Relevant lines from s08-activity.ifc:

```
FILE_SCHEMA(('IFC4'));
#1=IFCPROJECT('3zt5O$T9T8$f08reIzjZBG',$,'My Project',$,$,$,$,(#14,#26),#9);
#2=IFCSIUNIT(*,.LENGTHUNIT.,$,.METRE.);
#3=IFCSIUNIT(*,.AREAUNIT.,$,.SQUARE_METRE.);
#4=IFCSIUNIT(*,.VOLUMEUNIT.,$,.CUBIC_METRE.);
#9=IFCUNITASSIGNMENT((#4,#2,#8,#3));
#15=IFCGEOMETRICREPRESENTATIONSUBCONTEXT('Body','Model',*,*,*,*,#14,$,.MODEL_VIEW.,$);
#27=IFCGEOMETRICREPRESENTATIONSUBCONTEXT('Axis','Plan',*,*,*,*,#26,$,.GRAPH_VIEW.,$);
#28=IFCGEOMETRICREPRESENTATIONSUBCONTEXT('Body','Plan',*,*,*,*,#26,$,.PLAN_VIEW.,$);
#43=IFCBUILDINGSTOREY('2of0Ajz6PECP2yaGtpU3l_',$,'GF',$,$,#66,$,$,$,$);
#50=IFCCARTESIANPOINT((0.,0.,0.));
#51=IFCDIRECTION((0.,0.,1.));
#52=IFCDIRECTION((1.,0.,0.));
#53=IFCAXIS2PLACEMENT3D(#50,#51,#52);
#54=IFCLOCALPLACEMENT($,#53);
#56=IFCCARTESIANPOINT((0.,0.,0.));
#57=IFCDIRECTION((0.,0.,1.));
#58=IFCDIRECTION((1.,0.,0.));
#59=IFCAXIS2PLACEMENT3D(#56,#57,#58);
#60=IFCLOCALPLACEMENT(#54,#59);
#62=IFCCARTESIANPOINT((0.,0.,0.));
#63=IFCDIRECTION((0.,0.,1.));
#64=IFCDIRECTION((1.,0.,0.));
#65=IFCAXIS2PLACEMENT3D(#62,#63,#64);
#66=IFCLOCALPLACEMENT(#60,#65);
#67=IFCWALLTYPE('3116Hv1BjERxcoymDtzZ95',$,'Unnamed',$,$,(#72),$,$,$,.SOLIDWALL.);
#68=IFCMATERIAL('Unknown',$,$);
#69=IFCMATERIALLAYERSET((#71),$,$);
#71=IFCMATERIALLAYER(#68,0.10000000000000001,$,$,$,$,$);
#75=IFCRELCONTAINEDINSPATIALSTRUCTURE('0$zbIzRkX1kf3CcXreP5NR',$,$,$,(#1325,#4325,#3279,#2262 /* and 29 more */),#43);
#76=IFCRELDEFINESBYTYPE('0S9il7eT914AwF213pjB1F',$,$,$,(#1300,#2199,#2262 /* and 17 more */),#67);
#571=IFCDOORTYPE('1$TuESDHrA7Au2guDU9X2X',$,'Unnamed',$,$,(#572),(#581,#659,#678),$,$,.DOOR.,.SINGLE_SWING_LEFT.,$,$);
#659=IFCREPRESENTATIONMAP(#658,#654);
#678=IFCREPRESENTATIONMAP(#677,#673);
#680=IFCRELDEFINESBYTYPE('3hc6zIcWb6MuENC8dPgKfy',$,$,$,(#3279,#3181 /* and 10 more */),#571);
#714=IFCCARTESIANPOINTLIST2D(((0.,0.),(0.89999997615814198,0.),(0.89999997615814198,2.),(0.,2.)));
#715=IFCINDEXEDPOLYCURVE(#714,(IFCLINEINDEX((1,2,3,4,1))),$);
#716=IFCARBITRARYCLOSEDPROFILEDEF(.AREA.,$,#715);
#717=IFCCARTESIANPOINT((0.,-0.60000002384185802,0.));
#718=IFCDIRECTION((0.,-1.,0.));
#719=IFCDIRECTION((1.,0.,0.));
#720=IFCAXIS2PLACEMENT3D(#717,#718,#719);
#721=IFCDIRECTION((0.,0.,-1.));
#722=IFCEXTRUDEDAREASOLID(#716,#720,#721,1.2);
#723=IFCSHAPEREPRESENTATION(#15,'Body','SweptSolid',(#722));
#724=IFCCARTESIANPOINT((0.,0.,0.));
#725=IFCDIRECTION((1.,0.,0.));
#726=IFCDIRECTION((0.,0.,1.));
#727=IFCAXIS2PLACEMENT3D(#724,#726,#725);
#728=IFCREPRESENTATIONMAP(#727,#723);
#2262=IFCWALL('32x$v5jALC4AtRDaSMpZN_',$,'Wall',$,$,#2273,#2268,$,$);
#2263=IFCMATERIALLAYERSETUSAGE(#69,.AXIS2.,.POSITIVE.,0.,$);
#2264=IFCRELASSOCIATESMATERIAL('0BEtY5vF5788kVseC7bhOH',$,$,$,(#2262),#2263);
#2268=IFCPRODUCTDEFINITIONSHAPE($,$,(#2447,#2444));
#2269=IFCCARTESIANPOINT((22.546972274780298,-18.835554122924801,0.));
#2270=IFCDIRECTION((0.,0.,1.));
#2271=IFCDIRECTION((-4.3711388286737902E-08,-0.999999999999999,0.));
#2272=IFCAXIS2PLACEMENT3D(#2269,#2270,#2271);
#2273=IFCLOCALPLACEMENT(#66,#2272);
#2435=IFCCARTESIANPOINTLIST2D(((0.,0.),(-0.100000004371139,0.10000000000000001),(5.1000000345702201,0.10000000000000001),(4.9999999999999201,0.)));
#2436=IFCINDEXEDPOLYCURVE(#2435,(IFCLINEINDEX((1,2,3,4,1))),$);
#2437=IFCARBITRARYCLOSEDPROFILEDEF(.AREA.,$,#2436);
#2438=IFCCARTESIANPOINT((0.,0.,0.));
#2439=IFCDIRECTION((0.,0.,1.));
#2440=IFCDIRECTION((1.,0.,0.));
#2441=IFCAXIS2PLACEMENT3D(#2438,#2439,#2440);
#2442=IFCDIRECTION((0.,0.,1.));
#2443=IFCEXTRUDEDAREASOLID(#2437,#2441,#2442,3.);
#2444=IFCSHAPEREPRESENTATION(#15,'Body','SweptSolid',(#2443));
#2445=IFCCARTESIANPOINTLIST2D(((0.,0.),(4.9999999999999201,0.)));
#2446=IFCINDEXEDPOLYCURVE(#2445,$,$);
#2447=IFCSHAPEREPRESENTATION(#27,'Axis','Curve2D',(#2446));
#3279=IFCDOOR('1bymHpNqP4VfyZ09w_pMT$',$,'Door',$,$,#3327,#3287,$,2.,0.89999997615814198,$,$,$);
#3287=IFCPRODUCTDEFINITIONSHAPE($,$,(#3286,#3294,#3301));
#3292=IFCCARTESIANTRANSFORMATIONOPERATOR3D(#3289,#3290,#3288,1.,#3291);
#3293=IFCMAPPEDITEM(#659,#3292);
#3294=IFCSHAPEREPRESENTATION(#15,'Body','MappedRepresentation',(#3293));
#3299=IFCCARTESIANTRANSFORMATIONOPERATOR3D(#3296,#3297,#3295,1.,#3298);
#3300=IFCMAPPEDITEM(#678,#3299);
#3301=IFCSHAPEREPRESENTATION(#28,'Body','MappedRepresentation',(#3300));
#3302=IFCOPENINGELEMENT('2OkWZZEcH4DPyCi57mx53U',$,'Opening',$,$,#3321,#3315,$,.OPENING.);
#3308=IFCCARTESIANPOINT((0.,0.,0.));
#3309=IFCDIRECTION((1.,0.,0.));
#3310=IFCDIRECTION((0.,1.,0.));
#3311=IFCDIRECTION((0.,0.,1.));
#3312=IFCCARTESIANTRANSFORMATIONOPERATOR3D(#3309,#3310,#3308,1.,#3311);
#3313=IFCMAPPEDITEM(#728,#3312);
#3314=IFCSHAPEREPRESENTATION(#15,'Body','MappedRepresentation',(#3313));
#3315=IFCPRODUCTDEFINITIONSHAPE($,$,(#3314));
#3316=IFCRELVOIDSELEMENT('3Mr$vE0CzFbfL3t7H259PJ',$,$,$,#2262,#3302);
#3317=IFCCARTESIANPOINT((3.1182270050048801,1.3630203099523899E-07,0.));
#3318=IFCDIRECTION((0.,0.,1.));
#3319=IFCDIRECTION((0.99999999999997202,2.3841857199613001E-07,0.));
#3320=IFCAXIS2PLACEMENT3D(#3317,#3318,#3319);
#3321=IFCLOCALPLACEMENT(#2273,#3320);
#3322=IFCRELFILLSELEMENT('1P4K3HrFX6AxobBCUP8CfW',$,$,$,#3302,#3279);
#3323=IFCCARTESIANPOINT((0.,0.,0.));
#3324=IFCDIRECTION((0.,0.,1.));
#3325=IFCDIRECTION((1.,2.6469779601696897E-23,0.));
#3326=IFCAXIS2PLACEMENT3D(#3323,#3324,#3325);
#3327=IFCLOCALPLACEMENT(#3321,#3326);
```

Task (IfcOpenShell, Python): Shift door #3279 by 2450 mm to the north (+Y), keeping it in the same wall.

```python
import ifcopenshell
import ifcopenshell.api.geometry
import ifcopenshell.util.placement

model = ifcopenshell.open("s08-activity.ifc")

door = model.by_guid("1bymHpNqP4VfyZ09w_pMT$")
opening = door.FillsVoids[0].RelatingOpeningElement
wall = opening.VoidsElements[0].RelatingBuildingElement

wall_matrix = ifcopenshell.util.placement.get_local_placement(wall.ObjectPlacement)
shift = wall_matrix[:3, 0] * -2.45
before = ifcopenshell.util.placement.get_local_placement(door.ObjectPlacement)[:3, 3].copy()

# The door is placed relative to its opening, so it follows when the opening moves.
matrix = ifcopenshell.util.placement.get_local_placement(opening.ObjectPlacement)
matrix[:3, 3] += shift
ifcopenshell.api.geometry.edit_object_placement(
    model, product=opening, matrix=matrix, is_si=False, should_transform_children=True
)

after = ifcopenshell.util.placement.get_local_placement(door.ObjectPlacement)[:3, 3]
print("door moved by", (after - before).round(3) + 0.0)

model.write("s08-activity_updated.ifc")
```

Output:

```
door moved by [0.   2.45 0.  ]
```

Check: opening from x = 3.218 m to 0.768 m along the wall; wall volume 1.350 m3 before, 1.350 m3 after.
